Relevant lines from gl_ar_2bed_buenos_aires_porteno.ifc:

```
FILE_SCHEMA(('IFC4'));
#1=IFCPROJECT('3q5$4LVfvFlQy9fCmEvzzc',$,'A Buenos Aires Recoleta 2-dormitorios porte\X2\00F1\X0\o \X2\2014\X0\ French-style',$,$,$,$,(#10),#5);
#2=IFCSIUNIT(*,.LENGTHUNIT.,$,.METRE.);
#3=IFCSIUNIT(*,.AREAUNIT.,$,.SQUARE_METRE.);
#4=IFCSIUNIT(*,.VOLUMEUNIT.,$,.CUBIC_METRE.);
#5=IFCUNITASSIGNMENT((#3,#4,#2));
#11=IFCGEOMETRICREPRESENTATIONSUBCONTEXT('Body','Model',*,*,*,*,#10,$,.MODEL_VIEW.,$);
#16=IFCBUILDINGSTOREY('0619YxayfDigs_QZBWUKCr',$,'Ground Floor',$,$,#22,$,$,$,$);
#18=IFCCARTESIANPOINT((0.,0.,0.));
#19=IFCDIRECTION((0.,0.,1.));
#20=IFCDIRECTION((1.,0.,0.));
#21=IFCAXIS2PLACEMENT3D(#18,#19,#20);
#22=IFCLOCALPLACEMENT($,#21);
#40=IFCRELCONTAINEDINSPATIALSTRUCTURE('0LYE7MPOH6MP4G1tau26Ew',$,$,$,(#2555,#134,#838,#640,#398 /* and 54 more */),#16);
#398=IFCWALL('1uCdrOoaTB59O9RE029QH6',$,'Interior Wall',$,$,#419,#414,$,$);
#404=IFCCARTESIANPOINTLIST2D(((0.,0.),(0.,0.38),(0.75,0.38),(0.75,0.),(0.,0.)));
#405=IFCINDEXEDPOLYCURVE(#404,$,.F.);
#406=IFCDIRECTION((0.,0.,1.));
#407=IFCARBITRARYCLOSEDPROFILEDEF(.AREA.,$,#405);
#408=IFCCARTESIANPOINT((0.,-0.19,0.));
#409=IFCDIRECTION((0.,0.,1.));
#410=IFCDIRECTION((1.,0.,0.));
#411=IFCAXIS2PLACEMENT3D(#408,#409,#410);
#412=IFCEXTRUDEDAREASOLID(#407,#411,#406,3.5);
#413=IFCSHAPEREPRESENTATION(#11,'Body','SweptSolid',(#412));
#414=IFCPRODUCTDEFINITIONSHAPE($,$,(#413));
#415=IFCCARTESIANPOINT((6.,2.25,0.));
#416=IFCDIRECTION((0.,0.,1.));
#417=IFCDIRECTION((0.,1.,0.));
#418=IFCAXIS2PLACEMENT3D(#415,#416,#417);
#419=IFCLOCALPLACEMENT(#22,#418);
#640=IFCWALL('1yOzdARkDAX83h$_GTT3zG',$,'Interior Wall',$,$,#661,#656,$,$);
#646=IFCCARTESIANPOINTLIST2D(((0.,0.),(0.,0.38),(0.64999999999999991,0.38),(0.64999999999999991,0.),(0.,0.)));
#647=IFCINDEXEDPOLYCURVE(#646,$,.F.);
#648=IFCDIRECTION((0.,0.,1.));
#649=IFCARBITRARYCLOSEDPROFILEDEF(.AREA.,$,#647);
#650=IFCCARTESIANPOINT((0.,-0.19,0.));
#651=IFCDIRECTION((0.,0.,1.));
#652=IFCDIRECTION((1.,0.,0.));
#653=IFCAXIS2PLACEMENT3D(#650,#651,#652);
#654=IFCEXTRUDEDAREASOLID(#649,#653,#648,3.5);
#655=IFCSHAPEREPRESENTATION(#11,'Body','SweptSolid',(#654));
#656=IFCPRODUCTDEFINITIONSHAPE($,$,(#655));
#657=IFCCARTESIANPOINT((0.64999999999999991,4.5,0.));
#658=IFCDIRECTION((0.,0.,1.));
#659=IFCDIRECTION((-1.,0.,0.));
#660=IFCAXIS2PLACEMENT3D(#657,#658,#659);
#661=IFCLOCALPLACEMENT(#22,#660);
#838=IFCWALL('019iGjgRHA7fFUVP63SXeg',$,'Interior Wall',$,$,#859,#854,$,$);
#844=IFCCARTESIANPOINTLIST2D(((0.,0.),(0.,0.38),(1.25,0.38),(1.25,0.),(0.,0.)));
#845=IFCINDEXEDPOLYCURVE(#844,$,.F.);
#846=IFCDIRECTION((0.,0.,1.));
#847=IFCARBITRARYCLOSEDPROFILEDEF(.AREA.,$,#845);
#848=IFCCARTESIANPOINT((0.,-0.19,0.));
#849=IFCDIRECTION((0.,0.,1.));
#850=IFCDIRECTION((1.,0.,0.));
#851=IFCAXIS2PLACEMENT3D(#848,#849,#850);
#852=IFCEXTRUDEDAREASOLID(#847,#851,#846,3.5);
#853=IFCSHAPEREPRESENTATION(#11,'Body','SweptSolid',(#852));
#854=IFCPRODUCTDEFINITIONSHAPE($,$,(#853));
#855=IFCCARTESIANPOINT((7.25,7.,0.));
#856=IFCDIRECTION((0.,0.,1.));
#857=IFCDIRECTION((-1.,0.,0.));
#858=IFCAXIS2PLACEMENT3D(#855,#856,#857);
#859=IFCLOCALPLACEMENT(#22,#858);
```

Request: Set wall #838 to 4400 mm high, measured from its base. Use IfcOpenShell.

```python
import ifcopenshell
import ifcopenshell.geom
import ifcopenshell.util.representation
import ifcopenshell.util.shape

model = ifcopenshell.open("gl_ar_2bed_buenos_aires_porteno.ifc")
settings = ifcopenshell.geom.settings()


def volume(element):
    """Net volume in cubic metres, openings subtracted."""
    shape = ifcopenshell.geom.create_shape(settings, element)
    return ifcopenshell.util.shape.get_volume(shape.geometry)


wall = model.by_guid("019iGjgRHA7fFUVP63SXeg")
before = volume(wall)

body = ifcopenshell.util.representation.get_representation(wall, "Model", "Body")
solid = body.Items[0]
old_height = solid.Depth
solid.Depth = 4.4
after = volume(wall)

print(f"height {old_height:g} -> {solid.Depth:g}, volume {before:.3f} -> {after:.3f} m3")

model.write("gl_ar_2bed_buenos_aires_porteno_rev.ifc")
```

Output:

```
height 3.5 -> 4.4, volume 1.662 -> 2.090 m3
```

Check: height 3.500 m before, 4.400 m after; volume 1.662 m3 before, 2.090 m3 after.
